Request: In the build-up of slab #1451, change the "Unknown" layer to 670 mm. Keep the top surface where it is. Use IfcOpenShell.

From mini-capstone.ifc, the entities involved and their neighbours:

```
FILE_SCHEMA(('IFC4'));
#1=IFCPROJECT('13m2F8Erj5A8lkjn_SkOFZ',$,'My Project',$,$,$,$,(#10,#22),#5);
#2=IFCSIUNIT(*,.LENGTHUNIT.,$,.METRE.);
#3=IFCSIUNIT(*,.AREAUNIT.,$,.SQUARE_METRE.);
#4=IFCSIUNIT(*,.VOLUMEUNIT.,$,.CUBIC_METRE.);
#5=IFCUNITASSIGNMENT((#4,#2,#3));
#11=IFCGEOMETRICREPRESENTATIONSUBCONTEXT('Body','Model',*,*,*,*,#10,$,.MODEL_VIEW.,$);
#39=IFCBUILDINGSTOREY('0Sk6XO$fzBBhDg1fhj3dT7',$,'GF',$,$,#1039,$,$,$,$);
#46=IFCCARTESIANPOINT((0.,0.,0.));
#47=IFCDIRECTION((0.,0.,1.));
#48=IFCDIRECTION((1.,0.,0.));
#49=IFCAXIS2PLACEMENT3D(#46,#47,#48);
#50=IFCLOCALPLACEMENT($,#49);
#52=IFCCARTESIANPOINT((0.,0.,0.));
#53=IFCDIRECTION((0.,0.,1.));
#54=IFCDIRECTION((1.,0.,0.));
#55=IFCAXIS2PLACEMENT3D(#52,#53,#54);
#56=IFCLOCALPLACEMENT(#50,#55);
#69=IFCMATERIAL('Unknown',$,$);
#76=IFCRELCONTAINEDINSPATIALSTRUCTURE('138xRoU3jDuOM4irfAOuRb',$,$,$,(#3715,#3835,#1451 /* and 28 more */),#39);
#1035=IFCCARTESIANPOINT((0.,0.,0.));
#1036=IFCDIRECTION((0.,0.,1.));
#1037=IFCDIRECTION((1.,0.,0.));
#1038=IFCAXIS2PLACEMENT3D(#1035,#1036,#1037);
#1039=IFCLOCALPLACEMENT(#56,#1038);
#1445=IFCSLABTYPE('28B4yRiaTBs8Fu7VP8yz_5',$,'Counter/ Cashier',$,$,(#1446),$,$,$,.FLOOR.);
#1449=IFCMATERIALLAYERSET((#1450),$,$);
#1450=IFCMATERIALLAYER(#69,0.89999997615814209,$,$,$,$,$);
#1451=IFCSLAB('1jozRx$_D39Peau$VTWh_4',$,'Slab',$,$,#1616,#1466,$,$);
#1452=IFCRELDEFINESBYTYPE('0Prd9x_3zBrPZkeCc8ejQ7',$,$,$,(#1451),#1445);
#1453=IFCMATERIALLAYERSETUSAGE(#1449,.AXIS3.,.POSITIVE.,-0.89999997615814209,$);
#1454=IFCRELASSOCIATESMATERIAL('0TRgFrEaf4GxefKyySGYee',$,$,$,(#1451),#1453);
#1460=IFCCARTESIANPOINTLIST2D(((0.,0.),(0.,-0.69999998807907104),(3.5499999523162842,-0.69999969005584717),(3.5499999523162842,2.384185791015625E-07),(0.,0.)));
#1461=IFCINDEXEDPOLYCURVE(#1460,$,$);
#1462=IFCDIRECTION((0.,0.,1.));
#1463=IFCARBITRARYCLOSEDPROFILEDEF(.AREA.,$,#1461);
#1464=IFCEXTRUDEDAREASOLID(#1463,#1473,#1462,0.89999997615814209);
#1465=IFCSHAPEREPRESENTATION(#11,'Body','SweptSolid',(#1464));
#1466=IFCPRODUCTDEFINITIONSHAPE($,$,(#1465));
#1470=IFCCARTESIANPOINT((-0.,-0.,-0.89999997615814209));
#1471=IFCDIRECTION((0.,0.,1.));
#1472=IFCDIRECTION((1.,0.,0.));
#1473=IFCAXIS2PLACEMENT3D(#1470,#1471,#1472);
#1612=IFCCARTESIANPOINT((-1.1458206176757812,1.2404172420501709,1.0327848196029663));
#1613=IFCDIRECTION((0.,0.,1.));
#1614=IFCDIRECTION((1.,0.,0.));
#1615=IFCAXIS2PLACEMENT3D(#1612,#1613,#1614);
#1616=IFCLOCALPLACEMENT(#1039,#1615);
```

```python
import ifcopenshell
import ifcopenshell.util.element
import ifcopenshell.util.representation
import ifcopenshell.util.unit

model = ifcopenshell.open("mini-capstone.ifc")
unit_scale = ifcopenshell.util.unit.calculate_unit_scale(model)

layer_set = model.by_id(1449)
layer = next(l for l in layer_set.MaterialLayers if l.Material and l.Material.Name == "Unknown")
change = 0.67 / unit_scale - layer.LayerThickness
layer.LayerThickness += change

# Geometry does not follow the layer set by itself.
slabs = [e for e in ifcopenshell.util.element.get_elements_by_material(model, layer_set) if e.is_a("IfcSlab")]
for slab in sorted(slabs, key=lambda e: e.id()):
    body = ifcopenshell.util.representation.get_representation(slab, "Model", "Body")
    solid = body.Items[0]
    old_depth = solid.Depth
    solid.Depth += change
    # Extruded upwards: lower the start of the extrusion so the top stays.
    x, y, z = solid.Position.Location.Coordinates
    solid.Position.Location = model.createIfcCartesianPoint((x, y, z - change))
    print(slab.id(), f"{old_depth:g} -> {solid.Depth:g}")

# The layers are counted up from the underside, which has moved.
for usage in {ifcopenshell.util.element.get_material(slab) for slab in slabs}:
    usage.OffsetFromReferenceLine -= change

model.write("mini-capstone_rev.ifc")
```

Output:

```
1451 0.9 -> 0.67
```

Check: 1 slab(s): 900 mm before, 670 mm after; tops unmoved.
